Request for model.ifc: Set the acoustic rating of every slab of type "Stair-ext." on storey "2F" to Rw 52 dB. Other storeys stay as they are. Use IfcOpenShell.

First a look at what the model holds.

```python
import ifcopenshell
import ifcopenshell.util.element

model = ifcopenshell.open("model.ifc")
print(model.schema)
storey = next(s for s in model.by_type("IfcBuildingStorey") if s.Name == "2F")
slabs = [e for e in ifcopenshell.util.element.get_decomposition(storey) if e.is_a("IfcSlab")]
seen = {}
for e in slabs:
    element_type = ifcopenshell.util.element.get_type(e)
    key = (element_type.Name if element_type != e and element_type else None, ifcopenshell.util.element.get_pset(e, "Pset_SlabCommon", "AcousticRating"))
    seen[key] = seen.get(key, 0) + 1
for (name, value), count in sorted(seen.items(), key=str):
    print(count, "x", name, "|", value)
```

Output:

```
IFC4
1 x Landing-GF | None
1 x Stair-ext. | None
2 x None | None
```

```python
import ifcopenshell
import ifcopenshell.api.pset
import ifcopenshell.util.element

model = ifcopenshell.open("model.ifc")

storey = next(s for s in model.by_type("IfcBuildingStorey") if s.Name == "2F")
slabs = [e for e in ifcopenshell.util.element.get_decomposition(storey) if e.is_a("IfcSlab")]

count = 0
for e in slabs:
    element_type = ifcopenshell.util.element.get_type(e)
    if element_type in (None, e) or element_type.Name != "Stair-ext.":
        continue
    # add_pset returns the element's existing set when there is one.
    pset = ifcopenshell.api.pset.add_pset(model, product=e, name="Pset_SlabCommon")
    ifcopenshell.api.pset.edit_pset(model, pset=pset, properties={"AcousticRating": "Rw 52 dB"})
    count += 1

print(count, "slabs updated")

model.write("model_v2.ifc")
```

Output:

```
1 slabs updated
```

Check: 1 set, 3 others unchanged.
